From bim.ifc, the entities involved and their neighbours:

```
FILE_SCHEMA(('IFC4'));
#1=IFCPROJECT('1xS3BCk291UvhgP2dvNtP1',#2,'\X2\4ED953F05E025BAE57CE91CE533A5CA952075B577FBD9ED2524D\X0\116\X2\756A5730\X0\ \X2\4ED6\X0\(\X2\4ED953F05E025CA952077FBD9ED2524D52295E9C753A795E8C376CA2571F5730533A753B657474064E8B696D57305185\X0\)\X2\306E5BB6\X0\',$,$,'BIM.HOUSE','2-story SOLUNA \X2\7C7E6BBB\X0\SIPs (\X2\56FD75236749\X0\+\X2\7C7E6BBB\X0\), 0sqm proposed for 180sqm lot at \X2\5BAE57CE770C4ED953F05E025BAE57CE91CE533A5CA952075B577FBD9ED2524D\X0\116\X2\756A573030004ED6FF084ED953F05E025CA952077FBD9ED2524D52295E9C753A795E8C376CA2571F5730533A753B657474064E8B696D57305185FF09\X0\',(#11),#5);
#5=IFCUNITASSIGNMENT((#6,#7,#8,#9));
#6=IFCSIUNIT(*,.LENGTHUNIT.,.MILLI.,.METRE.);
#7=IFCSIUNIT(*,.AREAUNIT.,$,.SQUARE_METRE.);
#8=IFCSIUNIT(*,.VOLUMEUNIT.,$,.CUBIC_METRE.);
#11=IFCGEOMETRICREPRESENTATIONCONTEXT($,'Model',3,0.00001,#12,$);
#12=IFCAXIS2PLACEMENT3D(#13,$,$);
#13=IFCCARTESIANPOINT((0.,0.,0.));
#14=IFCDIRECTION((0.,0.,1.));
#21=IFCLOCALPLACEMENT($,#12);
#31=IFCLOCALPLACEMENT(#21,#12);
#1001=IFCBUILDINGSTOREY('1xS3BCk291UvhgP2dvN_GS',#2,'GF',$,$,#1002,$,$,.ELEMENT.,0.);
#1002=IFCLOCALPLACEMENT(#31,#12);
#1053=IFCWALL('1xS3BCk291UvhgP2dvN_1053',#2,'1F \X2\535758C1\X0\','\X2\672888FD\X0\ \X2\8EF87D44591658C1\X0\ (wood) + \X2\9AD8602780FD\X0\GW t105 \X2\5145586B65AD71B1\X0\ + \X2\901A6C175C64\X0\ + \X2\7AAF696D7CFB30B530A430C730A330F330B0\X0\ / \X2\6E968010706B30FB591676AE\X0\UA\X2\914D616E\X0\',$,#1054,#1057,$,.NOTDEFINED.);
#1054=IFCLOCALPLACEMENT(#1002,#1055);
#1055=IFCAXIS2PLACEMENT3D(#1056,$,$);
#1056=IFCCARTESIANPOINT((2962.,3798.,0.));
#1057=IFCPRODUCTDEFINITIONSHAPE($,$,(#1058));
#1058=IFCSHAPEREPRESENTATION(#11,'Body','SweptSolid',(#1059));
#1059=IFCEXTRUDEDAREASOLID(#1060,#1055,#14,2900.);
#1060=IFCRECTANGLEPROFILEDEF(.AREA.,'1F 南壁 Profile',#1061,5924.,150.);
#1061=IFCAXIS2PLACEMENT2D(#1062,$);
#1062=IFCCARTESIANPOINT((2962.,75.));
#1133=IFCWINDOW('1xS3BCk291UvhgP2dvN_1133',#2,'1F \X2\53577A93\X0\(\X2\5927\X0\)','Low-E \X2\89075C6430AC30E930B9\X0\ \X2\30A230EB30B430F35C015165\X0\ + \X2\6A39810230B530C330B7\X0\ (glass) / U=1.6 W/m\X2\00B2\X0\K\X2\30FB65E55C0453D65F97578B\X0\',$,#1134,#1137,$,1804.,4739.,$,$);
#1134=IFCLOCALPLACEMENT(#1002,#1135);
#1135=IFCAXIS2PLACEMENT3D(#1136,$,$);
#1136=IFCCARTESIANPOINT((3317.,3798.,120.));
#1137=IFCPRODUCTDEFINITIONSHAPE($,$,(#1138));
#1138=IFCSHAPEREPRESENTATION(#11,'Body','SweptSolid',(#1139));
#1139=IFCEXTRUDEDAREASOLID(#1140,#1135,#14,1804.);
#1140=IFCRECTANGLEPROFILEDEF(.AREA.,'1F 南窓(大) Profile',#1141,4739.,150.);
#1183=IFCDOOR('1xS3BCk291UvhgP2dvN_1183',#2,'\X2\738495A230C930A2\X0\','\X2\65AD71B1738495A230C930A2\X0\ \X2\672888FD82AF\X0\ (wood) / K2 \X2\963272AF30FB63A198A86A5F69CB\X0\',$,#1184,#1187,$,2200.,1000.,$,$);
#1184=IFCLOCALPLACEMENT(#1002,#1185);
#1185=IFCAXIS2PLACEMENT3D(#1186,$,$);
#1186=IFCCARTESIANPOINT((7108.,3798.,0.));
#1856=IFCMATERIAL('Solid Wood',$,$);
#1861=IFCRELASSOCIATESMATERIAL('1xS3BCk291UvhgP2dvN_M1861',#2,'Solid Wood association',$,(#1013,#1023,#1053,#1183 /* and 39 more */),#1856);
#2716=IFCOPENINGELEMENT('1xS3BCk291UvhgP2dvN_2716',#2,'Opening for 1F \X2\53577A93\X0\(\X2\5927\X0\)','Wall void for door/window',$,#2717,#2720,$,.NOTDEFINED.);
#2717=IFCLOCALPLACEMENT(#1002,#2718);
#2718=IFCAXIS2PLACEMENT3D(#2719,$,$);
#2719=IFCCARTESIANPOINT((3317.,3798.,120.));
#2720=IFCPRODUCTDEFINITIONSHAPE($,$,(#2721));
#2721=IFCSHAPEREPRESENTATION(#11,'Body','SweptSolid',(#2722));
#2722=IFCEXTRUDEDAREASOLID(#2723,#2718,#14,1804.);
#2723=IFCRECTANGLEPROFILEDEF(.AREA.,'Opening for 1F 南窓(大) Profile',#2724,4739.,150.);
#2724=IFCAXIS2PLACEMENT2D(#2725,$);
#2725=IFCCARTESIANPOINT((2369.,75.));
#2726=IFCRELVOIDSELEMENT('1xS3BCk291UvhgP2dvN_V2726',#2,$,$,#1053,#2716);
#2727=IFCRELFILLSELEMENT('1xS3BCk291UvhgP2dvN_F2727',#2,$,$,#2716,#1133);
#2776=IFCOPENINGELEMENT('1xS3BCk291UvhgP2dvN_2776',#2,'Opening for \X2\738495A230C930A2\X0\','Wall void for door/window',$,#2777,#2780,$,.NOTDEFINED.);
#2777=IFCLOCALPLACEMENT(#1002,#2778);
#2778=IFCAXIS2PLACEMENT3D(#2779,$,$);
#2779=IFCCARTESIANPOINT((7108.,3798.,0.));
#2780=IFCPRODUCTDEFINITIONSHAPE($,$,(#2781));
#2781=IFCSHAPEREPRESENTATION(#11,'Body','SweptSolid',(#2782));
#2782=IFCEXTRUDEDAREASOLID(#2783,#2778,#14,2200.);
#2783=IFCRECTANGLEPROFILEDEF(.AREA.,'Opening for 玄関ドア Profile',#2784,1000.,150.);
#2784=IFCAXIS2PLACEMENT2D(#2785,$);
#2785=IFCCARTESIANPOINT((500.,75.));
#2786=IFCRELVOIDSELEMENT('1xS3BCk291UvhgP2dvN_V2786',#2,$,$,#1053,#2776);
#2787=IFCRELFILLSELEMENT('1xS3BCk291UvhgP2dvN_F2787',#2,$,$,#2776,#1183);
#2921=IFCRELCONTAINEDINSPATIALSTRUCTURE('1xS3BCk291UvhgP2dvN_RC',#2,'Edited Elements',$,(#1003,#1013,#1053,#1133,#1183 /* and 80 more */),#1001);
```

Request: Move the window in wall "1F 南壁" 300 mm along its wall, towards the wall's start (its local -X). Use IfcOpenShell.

```python
import ifcopenshell
import ifcopenshell.api.geometry
import ifcopenshell.util.placement

model = ifcopenshell.open("bim.ifc")

window = model.by_guid("1xS3BCk291UvhgP2dvN_1133")
opening = window.FillsVoids[0].RelatingOpeningElement
wall = opening.VoidsElements[0].RelatingBuildingElement

wall_matrix = ifcopenshell.util.placement.get_local_placement(wall.ObjectPlacement)
shift = wall_matrix[:3, 0] * -300.0
before = ifcopenshell.util.placement.get_local_placement(window.ObjectPlacement)[:3, 3].copy()

# The window is not placed relative to its opening, so move both.
for product in (opening, window):
    matrix = ifcopenshell.util.placement.get_local_placement(product.ObjectPlacement)
    matrix[:3, 3] += shift
    ifcopenshell.api.geometry.edit_object_placement(model, product=product, matrix=matrix, is_si=False)

after = ifcopenshell.util.placement.get_local_placement(window.ObjectPlacement)[:3, 3]
print("window moved by", (after - before).round(3) + 0.0)

model.write("bim_rev.ifc")
```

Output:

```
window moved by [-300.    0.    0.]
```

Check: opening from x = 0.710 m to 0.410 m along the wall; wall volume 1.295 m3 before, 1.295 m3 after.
